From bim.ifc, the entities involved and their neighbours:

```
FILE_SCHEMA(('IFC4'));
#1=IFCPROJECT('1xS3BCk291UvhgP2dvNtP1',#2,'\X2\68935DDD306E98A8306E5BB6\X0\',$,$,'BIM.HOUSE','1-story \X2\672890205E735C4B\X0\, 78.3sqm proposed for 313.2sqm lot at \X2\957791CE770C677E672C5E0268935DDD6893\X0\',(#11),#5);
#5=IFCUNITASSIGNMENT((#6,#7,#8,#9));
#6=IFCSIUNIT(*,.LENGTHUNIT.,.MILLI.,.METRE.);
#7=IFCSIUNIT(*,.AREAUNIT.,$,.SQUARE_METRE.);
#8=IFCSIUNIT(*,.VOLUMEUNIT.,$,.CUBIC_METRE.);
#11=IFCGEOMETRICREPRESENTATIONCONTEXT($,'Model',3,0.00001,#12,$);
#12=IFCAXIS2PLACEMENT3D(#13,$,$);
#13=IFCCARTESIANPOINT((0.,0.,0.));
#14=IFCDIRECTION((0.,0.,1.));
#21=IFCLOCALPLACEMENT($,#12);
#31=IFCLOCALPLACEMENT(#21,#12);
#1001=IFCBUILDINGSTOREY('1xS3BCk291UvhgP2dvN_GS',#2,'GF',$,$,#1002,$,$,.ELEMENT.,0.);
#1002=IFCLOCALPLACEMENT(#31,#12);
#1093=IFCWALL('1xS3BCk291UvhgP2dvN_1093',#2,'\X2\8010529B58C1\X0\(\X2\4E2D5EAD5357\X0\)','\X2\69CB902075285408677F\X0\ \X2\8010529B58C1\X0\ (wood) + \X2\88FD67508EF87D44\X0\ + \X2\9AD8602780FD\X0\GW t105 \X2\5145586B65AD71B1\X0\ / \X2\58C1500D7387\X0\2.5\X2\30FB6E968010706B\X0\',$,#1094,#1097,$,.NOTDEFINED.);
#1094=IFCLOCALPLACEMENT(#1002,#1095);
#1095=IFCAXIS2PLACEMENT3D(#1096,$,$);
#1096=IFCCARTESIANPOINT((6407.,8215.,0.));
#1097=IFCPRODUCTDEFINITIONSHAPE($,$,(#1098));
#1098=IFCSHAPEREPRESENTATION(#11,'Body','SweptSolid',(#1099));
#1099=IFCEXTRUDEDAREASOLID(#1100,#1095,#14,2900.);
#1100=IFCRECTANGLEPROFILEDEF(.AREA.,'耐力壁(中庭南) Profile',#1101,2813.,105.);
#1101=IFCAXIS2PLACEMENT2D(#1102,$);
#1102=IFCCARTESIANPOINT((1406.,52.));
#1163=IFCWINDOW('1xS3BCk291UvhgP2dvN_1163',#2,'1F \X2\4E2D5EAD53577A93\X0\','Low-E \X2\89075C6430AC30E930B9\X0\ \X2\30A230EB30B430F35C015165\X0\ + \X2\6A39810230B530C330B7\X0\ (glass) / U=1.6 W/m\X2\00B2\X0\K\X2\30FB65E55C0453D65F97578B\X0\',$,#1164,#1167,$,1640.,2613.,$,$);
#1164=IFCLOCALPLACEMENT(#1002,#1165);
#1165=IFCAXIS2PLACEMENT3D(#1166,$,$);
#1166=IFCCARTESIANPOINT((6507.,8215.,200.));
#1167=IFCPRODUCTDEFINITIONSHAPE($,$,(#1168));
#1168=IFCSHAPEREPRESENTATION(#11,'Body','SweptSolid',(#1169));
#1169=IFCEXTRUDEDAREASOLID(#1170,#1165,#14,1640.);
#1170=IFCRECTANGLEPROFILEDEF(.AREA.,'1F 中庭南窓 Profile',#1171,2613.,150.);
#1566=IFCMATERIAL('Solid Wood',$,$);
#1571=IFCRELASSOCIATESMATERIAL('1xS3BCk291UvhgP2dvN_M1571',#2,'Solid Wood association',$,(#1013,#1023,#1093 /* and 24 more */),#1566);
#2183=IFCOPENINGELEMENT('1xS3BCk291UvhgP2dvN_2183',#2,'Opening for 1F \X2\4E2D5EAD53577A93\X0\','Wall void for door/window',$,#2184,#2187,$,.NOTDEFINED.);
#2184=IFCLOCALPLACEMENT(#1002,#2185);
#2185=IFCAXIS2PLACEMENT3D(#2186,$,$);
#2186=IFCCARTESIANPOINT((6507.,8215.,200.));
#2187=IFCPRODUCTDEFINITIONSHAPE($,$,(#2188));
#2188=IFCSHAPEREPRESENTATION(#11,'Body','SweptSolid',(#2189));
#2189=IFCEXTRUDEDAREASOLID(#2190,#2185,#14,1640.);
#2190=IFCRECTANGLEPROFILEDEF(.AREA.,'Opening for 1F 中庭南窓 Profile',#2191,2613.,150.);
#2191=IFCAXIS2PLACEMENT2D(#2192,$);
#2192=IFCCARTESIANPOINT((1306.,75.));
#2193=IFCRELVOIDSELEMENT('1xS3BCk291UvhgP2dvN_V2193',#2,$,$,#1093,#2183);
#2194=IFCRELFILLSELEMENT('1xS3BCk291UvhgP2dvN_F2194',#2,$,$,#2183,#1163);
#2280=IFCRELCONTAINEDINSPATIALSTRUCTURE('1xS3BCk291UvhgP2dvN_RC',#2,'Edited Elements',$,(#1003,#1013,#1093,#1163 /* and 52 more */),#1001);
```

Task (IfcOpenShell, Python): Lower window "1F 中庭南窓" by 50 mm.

```python
import numpy as np
import ifcopenshell
import ifcopenshell.api.geometry
import ifcopenshell.util.placement
import ifcopenshell.util.unit

model = ifcopenshell.open("bim.ifc")
unit_scale = ifcopenshell.util.unit.calculate_unit_scale(model)

window = model.by_guid("1xS3BCk291UvhgP2dvN_1163")
opening = window.FillsVoids[0].RelatingOpeningElement
dz = -0.05 / unit_scale

shift = np.array([0.0, 0.0, dz])
# The window is not placed relative to its opening, so move both.
for product in (opening, window):
    matrix = ifcopenshell.util.placement.get_local_placement(product.ObjectPlacement)
    matrix[:3, 3] += shift
    ifcopenshell.api.geometry.edit_object_placement(model, product=product, matrix=matrix, is_si=False)

print(f"moved by {dz * unit_scale:+.3f} m")

model.write("bim_v2.ifc")
```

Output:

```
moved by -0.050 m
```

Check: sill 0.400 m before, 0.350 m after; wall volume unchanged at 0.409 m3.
